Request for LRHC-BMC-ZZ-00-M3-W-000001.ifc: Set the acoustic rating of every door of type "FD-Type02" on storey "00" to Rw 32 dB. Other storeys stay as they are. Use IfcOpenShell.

First a look at what the model holds.

```python
import ifcopenshell
import ifcopenshell.util.element

model = ifcopenshell.open("LRHC-BMC-ZZ-00-M3-W-000001.ifc")
print(model.schema)
storey = next(s for s in model.by_type("IfcBuildingStorey") if s.Name == "00")
doors = [e for e in ifcopenshell.util.element.get_decomposition(storey) if e.is_a("IfcDoor")]
seen = {}
for e in doors:
    element_type = ifcopenshell.util.element.get_type(e)
    key = (element_type.Name if element_type != e and element_type else None, ifcopenshell.util.element.get_pset(e, "Pset_DoorCommon", "AcousticRating"))
    seen[key] = seen.get(key, 0) + 1
for (name, value), count in sorted(seen.items(), key=str):
    print(count, "x", name, "|", value)
```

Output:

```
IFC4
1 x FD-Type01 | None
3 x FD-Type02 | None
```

```python
import ifcopenshell
import ifcopenshell.api.pset
import ifcopenshell.util.element

model = ifcopenshell.open("LRHC-BMC-ZZ-00-M3-W-000001.ifc")

storey = next(s for s in model.by_type("IfcBuildingStorey") if s.Name == "00")
doors = [e for e in ifcopenshell.util.element.get_decomposition(storey) if e.is_a("IfcDoor")]

count = 0
for e in doors:
    element_type = ifcopenshell.util.element.get_type(e)
    if element_type in (None, e) or element_type.Name != "FD-Type02":
        continue
    # add_pset returns the element's existing set when there is one.
    pset = ifcopenshell.api.pset.add_pset(model, product=e, name="Pset_DoorCommon")
    ifcopenshell.api.pset.edit_pset(model, pset=pset, properties={"AcousticRating": "Rw 32 dB"})
    count += 1

print(count, "doors updated")

model.write("LRHC-BMC-ZZ-00-M3-W-000001_rev.ifc")
```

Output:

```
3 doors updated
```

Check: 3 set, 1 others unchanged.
